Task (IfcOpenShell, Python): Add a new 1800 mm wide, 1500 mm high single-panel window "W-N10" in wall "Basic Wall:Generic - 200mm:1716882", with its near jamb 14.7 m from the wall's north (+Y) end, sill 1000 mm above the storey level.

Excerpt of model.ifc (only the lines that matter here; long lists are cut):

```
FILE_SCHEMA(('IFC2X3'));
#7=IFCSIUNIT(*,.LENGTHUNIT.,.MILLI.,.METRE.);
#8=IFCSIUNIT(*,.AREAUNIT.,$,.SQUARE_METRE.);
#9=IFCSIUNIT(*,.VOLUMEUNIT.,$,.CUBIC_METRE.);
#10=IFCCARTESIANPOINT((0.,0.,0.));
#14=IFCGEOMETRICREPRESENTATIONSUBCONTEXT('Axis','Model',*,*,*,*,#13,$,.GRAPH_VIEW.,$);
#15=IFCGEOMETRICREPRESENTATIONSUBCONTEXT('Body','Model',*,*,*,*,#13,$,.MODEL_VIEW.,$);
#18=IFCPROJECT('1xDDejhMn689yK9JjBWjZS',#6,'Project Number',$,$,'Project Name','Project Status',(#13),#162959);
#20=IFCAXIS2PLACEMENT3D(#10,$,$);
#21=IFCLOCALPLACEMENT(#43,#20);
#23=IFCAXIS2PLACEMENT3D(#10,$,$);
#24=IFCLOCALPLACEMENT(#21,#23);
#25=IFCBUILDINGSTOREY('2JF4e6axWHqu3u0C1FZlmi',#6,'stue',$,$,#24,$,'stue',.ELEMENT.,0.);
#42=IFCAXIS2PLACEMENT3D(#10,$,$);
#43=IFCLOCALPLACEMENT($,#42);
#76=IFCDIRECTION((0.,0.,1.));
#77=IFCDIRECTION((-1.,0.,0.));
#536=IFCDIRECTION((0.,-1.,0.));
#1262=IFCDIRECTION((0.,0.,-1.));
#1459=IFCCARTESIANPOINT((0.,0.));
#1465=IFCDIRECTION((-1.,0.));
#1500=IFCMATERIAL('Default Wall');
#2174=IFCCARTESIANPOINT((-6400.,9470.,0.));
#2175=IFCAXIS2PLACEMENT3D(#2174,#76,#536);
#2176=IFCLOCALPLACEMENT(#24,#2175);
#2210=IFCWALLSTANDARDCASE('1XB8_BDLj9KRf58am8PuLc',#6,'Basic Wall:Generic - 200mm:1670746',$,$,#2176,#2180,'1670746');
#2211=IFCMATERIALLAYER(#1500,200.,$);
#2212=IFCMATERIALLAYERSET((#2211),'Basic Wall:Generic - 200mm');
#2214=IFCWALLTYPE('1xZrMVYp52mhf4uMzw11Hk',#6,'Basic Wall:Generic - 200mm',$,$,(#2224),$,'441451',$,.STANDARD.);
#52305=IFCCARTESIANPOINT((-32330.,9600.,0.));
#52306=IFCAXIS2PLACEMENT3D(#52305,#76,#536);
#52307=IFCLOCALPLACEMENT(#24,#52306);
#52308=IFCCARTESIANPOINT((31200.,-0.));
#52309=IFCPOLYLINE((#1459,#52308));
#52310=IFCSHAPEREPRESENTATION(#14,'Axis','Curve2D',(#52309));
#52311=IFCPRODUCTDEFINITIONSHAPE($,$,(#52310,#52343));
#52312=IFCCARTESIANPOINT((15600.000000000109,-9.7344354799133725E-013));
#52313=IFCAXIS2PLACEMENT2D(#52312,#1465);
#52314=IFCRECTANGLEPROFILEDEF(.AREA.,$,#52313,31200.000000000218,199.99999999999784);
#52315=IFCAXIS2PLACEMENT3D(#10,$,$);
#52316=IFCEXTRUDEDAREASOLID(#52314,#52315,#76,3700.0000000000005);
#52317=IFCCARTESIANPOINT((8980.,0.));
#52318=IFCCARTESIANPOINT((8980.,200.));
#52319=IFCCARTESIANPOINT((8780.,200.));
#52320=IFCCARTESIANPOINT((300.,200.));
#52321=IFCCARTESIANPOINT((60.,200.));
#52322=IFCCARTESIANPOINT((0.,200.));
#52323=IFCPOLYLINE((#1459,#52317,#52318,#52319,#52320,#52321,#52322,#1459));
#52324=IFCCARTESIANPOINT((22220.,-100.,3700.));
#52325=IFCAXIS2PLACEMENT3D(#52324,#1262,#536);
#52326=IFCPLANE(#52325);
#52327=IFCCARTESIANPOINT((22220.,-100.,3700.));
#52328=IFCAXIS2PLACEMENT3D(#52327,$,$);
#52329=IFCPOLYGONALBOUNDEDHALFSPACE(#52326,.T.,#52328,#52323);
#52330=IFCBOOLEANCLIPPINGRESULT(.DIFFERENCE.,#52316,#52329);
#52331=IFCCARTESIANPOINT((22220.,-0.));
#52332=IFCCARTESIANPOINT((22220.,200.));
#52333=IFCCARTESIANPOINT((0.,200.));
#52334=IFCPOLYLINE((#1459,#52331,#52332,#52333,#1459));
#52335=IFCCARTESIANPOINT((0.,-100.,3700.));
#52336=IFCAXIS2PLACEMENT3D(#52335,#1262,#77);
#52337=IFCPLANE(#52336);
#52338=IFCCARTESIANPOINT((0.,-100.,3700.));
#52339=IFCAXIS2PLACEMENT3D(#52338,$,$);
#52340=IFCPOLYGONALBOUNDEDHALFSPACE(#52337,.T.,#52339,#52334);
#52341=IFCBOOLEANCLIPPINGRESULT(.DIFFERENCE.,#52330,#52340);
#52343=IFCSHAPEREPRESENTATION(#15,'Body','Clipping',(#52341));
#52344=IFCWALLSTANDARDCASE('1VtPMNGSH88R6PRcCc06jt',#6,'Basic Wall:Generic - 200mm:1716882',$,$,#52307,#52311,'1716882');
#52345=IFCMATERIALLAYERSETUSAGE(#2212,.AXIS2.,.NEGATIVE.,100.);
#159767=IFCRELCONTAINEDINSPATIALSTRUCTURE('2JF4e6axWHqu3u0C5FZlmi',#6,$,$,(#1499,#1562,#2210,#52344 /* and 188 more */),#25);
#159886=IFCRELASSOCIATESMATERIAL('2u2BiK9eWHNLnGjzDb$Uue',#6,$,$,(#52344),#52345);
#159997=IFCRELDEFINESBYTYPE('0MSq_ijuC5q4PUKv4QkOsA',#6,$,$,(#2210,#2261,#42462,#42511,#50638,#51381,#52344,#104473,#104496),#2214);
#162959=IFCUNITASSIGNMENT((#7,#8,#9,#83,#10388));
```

```python
import numpy as np
import ifcopenshell
import ifcopenshell.api.feature
import ifcopenshell.api.geometry
import ifcopenshell.api.root
import ifcopenshell.api.spatial
import ifcopenshell.api.type
import ifcopenshell.geom
import ifcopenshell.util.element
import ifcopenshell.util.placement
import ifcopenshell.util.representation
import ifcopenshell.util.shape
import ifcopenshell.util.unit

model = ifcopenshell.open("model.ifc")
unit_scale = ifcopenshell.util.unit.calculate_unit_scale(model)
settings = ifcopenshell.geom.settings()


def volume(element):
    """Net volume in cubic metres, openings subtracted."""
    shape = ifcopenshell.geom.create_shape(settings, element)
    return ifcopenshell.util.shape.get_volume(shape.geometry)


wall = model.by_guid("1VtPMNGSH88R6PRcCc06jt")
storey = ifcopenshell.util.element.get_container(wall, ifc_class="IfcBuildingStorey")
context = ifcopenshell.util.representation.get_context(model, "Model", "Body", "MODEL_VIEW")
before = volume(wall)

width, height, from_end, sill = 1.8, 1.5, 14.7, 1  # metres

# The wall runs along its own X axis, and the end named is its -X end.
wall_shape = ifcopenshell.geom.create_shape(settings, wall)
x, y, z = ifcopenshell.util.shape.get_vertices(wall_shape.geometry).T
start = x.min() + from_end
face, thickness = float(y.min()), float(y.max() - y.min())
wall_matrix = ifcopenshell.util.placement.get_local_placement(wall.ObjectPlacement)
level = ifcopenshell.util.placement.get_local_placement(storey.ObjectPlacement)[2, 3]


def in_wall(x, y):
    """Placement at x, y metres in the wall's axes, at sill height."""
    matrix = wall_matrix.copy()
    matrix[:, 3] = wall_matrix @ np.array([x / unit_scale, y / unit_scale, 0.0, 1.0])
    matrix[2, 3] = level + sill / unit_scale
    return matrix


# Opening: a box that overshoots both wall faces by 50 mm.
opening = ifcopenshell.api.root.create_entity(model, ifc_class="IfcOpeningElement")
box = ifcopenshell.api.geometry.add_wall_representation(
    model, context=context, length=width, height=height, thickness=thickness + 0.1
)
ifcopenshell.api.geometry.assign_representation(model, product=opening, representation=box)
ifcopenshell.api.geometry.edit_object_placement(model, product=opening, matrix=in_wall(start, face - 0.05), is_si=False)
ifcopenshell.api.feature.add_feature(model, feature=opening, element=wall)

window = ifcopenshell.api.root.create_entity(model, ifc_class="IfcWindow", name="W-N10")
window.OverallWidth, window.OverallHeight = width / unit_scale, height / unit_scale
body = ifcopenshell.api.geometry.add_window_representation(
    model,
    context=context,
    overall_width=window.OverallWidth,
    overall_height=window.OverallHeight,
    partition_type="SINGLE_PANEL",
)
ifcopenshell.api.geometry.assign_representation(model, product=window, representation=body)
ifcopenshell.api.spatial.assign_container(model, products=[window], relating_structure=storey)
fills = ifcopenshell.api.feature.add_filling(model, opening=opening, element=window)
fills.OwnerHistory = window.OwnerHistory  # required in IFC2X3

# IFC2X3 keeps the operation on the window style.
style = ifcopenshell.api.root.create_entity(model, ifc_class="IfcWindowStyle", name="W-N10")
style.OperationType, style.ConstructionType = "SINGLE_PANEL", "NOTDEFINED"
style.ParameterTakesPrecedence = style.Sizeable = False
ifcopenshell.api.type.assign_type(model, related_objects=[window], relating_type=style)

# Centre the window in the wall's thickness.
ifcopenshell.api.geometry.edit_object_placement(model, product=window, matrix=in_wall(start, face), is_si=False)
window_shape = ifcopenshell.geom.create_shape(settings, window)
depth = ifcopenshell.util.shape.get_vertices(window_shape.geometry)[:, 1]
offset = face + thickness / 2 - (depth.min() + depth.max()) / 2
ifcopenshell.api.geometry.edit_object_placement(model, product=window, matrix=in_wall(start, offset), is_si=False)

after = volume(wall)

print(f"wall volume {before:.3f} -> {after:.3f} m3")

model.write("model_updated.ifc")
```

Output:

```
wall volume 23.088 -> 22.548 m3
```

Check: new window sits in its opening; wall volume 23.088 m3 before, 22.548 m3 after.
